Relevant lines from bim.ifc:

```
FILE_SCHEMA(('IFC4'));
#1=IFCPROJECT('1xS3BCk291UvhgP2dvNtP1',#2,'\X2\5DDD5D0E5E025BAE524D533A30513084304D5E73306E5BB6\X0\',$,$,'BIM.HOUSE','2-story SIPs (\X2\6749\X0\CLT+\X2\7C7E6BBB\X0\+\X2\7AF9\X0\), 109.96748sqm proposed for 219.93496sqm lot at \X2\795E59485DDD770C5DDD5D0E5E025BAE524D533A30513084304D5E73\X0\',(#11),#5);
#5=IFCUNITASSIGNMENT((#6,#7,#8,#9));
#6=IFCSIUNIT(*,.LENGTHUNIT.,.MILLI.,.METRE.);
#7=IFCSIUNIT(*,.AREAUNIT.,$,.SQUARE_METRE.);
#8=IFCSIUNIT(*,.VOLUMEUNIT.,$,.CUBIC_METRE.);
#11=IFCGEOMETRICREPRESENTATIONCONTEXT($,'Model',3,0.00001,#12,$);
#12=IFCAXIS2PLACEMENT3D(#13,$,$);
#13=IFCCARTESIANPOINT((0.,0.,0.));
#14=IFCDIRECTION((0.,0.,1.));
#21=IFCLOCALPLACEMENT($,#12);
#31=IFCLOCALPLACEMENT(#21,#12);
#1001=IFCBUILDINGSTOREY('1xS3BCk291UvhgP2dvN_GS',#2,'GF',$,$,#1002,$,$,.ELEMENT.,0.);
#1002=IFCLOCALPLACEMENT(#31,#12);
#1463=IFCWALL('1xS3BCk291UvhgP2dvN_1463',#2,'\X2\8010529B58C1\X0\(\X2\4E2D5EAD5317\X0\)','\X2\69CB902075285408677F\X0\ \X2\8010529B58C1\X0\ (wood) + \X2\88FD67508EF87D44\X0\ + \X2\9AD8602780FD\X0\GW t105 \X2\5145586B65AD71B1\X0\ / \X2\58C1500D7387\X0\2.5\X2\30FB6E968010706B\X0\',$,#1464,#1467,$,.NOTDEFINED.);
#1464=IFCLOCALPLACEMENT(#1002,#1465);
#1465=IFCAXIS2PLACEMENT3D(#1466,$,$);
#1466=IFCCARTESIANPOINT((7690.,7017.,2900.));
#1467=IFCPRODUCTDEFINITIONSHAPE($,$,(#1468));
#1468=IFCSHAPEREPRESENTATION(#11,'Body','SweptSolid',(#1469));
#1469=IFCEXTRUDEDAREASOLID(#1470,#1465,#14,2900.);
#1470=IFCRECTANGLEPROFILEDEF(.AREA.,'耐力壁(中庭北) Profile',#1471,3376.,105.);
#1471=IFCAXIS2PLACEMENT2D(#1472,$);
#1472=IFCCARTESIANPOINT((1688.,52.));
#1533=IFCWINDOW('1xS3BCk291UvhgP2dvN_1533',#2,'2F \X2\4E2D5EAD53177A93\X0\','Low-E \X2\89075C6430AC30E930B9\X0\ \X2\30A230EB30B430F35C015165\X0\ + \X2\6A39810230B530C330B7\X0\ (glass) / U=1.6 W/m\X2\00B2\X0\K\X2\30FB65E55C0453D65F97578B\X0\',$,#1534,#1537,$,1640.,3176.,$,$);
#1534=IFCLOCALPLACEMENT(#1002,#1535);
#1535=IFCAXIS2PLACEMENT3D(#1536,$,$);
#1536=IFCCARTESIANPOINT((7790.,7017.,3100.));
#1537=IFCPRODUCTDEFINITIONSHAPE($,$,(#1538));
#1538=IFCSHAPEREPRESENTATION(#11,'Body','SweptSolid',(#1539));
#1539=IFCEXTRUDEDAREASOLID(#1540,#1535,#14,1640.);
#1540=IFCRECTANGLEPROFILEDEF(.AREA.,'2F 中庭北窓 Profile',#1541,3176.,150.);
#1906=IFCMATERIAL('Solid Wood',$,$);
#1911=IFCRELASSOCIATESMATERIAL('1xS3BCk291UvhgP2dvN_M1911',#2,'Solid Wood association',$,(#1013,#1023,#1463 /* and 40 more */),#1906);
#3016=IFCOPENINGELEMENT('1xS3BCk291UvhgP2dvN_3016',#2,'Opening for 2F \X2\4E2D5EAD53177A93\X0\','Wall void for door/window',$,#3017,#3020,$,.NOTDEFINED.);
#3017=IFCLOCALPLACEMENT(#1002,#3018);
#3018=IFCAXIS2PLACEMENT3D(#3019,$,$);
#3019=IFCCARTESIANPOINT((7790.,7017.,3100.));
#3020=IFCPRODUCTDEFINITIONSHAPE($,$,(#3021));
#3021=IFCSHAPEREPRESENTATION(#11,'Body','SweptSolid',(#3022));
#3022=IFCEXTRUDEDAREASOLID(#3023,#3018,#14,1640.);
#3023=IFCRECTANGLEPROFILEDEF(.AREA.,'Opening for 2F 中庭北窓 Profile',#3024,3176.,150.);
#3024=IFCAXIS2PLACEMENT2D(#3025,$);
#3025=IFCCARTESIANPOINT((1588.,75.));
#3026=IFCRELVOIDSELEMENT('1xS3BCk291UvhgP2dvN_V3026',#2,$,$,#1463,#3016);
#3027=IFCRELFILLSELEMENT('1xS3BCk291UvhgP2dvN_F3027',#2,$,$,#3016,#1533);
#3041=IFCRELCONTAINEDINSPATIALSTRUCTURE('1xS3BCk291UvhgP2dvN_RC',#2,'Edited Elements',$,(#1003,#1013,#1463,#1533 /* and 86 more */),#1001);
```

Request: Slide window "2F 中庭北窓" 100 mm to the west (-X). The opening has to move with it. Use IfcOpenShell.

```python
import ifcopenshell
import ifcopenshell.api.geometry
import ifcopenshell.util.placement

model = ifcopenshell.open("bim.ifc")

window = model.by_guid("1xS3BCk291UvhgP2dvN_1533")
opening = window.FillsVoids[0].RelatingOpeningElement
wall = opening.VoidsElements[0].RelatingBuildingElement

wall_matrix = ifcopenshell.util.placement.get_local_placement(wall.ObjectPlacement)
shift = wall_matrix[:3, 0] * -100.0
before = ifcopenshell.util.placement.get_local_placement(window.ObjectPlacement)[:3, 3].copy()

# The window is not placed relative to its opening, so move both.
for product in (opening, window):
    matrix = ifcopenshell.util.placement.get_local_placement(product.ObjectPlacement)
    matrix[:3, 3] += shift
    ifcopenshell.api.geometry.edit_object_placement(model, product=product, matrix=matrix, is_si=False)

after = ifcopenshell.util.placement.get_local_placement(window.ObjectPlacement)[:3, 3]
print("window moved by", (after - before).round(3) + 0.0)

model.write("bim_rev.ifc")
```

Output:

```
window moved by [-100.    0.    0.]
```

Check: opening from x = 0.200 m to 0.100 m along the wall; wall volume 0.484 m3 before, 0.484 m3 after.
